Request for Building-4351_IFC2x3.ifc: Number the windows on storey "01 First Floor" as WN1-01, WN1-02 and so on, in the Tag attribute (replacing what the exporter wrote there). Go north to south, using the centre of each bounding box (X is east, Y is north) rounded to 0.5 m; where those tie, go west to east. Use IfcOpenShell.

First a look at what the model holds.

```python
import ifcopenshell
import ifcopenshell.util.element
import ifcopenshell.util.placement

model = ifcopenshell.open("Building-4351_IFC2x3.ifc")
print(model.schema)
storey = next(s for s in model.by_type("IfcBuildingStorey") if s.Name == "01 First Floor")
windows = [e for e in ifcopenshell.util.element.get_decomposition(storey) if e.is_a("IfcWindow")]
for e in sorted(windows, key=lambda e: e.id()):
    origin = ifcopenshell.util.placement.get_local_placement(e.ObjectPlacement)[:3, 3]
    print(e.id(), e.Tag, e.Name, origin.round(2) + 0.0, sep=" | ")
```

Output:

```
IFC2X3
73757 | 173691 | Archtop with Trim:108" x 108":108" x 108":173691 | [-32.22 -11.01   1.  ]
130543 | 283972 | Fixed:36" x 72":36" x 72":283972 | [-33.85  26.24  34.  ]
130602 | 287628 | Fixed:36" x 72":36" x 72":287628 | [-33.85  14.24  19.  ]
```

```python
import ifcopenshell
import ifcopenshell.geom
import ifcopenshell.util.element
import ifcopenshell.util.shape

model = ifcopenshell.open("Building-4351_IFC2x3.ifc")
settings = ifcopenshell.geom.settings()
settings.set("use-world-coords", True)


def centre(element):
    shape = ifcopenshell.geom.create_shape(settings, element)
    return ifcopenshell.util.shape.get_bbox_centroid(shape.geometry)


storey = next(s for s in model.by_type("IfcBuildingStorey") if s.Name == "01 First Floor")
windows = [e for e in ifcopenshell.util.element.get_decomposition(storey) if e.is_a("IfcWindow")]

# Insertion points can sit at a corner or the storey origin, so sort by the geometry (in metres).
centres = {e: centre(e) for e in windows}
windows.sort(key=lambda e: (-round(centres[e][1] / 0.5), centres[e][0]))

for i, e in enumerate(windows, start=1):
    number = f"WN1-{i:02d}"
    e.Tag = number
    print(e.id(), number)

model.write("Building-4351_IFC2x3_updated.ifc")
```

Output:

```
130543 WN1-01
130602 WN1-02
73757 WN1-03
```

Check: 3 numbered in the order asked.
